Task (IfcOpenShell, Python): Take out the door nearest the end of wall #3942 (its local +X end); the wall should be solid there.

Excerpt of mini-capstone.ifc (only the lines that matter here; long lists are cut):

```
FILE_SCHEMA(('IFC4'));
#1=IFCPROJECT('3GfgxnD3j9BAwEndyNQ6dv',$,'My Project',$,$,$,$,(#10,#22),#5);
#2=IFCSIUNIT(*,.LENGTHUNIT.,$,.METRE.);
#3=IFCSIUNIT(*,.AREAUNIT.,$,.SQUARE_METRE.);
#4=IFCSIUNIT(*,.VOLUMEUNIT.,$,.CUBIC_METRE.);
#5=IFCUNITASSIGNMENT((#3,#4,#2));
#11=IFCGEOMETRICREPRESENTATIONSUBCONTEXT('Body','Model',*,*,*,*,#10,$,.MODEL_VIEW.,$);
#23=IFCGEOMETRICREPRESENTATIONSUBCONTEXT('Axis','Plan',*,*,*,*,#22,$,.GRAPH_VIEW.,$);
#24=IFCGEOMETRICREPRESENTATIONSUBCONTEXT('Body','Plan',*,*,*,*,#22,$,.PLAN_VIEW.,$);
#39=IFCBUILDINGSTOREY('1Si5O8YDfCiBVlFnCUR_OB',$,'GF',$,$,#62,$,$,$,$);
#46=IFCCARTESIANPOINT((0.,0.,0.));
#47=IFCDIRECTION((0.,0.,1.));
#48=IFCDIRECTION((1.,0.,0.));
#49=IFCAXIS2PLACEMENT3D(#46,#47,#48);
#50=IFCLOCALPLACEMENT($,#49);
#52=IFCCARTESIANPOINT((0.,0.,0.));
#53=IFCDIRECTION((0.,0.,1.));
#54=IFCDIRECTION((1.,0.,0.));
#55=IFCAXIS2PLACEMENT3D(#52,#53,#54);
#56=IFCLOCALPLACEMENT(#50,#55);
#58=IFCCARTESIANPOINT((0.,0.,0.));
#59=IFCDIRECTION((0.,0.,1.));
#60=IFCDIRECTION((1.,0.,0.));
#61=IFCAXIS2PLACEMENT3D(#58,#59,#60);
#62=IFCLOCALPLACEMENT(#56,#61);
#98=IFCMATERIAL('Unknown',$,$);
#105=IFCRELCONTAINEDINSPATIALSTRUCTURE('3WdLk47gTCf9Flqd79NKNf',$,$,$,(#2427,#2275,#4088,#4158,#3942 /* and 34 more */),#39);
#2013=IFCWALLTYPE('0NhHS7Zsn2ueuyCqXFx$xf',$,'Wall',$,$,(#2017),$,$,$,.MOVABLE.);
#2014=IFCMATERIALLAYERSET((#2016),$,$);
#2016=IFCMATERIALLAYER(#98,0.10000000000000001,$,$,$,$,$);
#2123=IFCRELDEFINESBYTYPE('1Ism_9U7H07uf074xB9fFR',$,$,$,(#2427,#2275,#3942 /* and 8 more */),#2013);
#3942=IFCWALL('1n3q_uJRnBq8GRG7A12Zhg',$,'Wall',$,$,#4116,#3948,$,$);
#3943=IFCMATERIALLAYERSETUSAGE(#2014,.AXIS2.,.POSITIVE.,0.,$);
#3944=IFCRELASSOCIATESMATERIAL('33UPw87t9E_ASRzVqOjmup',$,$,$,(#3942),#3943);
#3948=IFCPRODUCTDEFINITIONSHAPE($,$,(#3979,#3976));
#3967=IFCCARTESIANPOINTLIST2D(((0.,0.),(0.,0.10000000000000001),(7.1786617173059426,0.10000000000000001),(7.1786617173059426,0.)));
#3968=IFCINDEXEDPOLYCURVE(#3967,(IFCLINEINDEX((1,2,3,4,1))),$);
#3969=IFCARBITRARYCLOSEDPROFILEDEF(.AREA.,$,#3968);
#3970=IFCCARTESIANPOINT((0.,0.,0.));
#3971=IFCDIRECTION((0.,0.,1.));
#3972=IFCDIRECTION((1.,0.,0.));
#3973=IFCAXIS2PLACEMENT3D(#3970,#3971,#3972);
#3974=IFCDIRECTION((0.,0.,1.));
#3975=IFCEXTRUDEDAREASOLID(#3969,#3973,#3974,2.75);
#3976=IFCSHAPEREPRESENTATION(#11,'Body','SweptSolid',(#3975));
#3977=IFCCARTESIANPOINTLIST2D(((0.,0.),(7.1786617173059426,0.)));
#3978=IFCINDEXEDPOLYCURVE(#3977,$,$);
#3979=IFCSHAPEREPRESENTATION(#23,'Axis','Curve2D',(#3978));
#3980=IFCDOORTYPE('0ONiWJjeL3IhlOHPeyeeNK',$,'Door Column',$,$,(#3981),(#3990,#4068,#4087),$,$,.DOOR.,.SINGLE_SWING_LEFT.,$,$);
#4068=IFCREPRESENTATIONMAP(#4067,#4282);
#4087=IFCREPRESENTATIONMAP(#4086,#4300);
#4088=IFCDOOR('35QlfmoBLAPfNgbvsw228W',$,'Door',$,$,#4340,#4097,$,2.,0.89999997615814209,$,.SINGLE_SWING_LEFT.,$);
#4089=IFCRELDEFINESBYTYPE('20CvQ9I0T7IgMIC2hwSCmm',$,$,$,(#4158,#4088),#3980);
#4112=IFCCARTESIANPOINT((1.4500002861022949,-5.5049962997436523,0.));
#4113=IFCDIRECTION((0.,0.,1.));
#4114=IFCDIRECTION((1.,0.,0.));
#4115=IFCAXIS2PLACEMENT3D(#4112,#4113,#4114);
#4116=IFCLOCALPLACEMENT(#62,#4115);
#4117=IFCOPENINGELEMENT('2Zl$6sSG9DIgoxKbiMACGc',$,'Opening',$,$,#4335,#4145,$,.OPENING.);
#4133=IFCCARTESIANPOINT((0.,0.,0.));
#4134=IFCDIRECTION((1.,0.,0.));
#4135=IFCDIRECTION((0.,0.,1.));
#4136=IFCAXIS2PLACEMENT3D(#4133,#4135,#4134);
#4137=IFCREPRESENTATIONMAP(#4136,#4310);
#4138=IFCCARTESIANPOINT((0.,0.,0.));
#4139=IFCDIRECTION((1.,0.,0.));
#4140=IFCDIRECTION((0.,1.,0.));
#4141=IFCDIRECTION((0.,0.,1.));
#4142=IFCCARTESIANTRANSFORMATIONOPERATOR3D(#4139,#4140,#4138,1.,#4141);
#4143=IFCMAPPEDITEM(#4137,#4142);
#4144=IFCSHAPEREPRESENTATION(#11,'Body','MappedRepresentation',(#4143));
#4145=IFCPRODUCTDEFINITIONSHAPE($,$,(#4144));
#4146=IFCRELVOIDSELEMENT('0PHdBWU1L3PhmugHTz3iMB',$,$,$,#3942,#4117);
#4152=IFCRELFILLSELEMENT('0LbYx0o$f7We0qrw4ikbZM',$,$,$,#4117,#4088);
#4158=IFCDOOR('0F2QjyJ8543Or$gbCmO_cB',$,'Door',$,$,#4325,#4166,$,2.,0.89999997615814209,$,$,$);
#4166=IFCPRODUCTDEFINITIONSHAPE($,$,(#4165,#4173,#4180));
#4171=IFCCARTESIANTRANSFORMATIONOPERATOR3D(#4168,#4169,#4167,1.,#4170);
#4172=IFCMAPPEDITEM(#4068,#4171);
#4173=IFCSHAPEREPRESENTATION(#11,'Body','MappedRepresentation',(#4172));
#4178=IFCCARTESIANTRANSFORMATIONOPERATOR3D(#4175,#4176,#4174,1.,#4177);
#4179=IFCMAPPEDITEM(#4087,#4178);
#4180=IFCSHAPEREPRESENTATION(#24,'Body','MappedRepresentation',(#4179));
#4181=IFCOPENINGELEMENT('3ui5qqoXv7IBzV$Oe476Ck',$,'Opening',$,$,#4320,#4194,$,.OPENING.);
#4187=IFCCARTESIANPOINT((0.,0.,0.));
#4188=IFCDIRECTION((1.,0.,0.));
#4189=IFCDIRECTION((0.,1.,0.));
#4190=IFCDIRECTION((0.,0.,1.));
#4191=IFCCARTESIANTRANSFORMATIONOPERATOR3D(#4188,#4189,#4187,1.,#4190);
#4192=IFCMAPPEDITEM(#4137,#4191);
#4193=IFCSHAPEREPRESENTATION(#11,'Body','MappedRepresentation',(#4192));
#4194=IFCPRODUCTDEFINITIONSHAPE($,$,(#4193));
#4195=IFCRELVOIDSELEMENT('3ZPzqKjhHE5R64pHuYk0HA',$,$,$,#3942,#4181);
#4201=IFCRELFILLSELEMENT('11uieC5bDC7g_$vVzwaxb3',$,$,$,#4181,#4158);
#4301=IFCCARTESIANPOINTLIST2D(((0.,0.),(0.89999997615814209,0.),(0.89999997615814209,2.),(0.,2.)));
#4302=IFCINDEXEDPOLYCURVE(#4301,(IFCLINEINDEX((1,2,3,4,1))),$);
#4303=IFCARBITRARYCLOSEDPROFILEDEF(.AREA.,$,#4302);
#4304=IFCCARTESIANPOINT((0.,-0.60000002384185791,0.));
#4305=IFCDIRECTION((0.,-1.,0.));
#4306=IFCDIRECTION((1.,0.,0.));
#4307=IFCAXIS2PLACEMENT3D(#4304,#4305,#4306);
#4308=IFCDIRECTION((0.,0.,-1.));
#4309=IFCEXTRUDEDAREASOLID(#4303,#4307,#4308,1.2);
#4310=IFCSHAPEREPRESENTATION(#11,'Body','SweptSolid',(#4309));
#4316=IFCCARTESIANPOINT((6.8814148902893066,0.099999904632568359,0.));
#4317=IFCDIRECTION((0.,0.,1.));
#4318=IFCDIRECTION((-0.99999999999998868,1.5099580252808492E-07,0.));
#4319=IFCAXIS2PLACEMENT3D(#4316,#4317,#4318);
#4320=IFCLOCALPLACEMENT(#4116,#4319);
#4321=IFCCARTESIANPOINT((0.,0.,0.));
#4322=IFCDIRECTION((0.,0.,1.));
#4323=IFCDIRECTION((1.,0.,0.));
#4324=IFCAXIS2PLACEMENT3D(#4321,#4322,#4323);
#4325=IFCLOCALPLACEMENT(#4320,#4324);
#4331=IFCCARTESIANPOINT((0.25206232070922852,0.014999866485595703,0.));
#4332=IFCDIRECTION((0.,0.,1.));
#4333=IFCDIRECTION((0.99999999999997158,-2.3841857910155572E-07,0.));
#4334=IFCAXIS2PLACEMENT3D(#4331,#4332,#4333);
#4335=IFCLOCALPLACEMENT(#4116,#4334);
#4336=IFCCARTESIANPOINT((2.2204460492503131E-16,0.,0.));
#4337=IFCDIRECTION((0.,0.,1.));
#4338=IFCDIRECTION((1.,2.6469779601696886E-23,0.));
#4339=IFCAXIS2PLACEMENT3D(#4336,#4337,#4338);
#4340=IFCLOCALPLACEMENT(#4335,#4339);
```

```python
import ifcopenshell
import ifcopenshell.api.feature
import ifcopenshell.api.root
import ifcopenshell.geom
import ifcopenshell.util.shape

model = ifcopenshell.open("mini-capstone.ifc")
settings = ifcopenshell.geom.settings()


def volume(element):
    """Net volume in cubic metres, openings subtracted."""
    shape = ifcopenshell.geom.create_shape(settings, element)
    return ifcopenshell.util.shape.get_volume(shape.geometry)


door = model.by_guid("0F2QjyJ8543Or$gbCmO_cB")
opening = door.FillsVoids[0].RelatingOpeningElement
wall = opening.VoidsElements[0].RelatingBuildingElement
before = volume(wall)

ifcopenshell.api.root.remove_product(model, product=door)
ifcopenshell.api.feature.remove_feature(model, feature=opening)

after = volume(wall)

print(f"wall volume {before:.3f} -> {after:.3f} m3")

model.write("mini-capstone_rev.ifc")
```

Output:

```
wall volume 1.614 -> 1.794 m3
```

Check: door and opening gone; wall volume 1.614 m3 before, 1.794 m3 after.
